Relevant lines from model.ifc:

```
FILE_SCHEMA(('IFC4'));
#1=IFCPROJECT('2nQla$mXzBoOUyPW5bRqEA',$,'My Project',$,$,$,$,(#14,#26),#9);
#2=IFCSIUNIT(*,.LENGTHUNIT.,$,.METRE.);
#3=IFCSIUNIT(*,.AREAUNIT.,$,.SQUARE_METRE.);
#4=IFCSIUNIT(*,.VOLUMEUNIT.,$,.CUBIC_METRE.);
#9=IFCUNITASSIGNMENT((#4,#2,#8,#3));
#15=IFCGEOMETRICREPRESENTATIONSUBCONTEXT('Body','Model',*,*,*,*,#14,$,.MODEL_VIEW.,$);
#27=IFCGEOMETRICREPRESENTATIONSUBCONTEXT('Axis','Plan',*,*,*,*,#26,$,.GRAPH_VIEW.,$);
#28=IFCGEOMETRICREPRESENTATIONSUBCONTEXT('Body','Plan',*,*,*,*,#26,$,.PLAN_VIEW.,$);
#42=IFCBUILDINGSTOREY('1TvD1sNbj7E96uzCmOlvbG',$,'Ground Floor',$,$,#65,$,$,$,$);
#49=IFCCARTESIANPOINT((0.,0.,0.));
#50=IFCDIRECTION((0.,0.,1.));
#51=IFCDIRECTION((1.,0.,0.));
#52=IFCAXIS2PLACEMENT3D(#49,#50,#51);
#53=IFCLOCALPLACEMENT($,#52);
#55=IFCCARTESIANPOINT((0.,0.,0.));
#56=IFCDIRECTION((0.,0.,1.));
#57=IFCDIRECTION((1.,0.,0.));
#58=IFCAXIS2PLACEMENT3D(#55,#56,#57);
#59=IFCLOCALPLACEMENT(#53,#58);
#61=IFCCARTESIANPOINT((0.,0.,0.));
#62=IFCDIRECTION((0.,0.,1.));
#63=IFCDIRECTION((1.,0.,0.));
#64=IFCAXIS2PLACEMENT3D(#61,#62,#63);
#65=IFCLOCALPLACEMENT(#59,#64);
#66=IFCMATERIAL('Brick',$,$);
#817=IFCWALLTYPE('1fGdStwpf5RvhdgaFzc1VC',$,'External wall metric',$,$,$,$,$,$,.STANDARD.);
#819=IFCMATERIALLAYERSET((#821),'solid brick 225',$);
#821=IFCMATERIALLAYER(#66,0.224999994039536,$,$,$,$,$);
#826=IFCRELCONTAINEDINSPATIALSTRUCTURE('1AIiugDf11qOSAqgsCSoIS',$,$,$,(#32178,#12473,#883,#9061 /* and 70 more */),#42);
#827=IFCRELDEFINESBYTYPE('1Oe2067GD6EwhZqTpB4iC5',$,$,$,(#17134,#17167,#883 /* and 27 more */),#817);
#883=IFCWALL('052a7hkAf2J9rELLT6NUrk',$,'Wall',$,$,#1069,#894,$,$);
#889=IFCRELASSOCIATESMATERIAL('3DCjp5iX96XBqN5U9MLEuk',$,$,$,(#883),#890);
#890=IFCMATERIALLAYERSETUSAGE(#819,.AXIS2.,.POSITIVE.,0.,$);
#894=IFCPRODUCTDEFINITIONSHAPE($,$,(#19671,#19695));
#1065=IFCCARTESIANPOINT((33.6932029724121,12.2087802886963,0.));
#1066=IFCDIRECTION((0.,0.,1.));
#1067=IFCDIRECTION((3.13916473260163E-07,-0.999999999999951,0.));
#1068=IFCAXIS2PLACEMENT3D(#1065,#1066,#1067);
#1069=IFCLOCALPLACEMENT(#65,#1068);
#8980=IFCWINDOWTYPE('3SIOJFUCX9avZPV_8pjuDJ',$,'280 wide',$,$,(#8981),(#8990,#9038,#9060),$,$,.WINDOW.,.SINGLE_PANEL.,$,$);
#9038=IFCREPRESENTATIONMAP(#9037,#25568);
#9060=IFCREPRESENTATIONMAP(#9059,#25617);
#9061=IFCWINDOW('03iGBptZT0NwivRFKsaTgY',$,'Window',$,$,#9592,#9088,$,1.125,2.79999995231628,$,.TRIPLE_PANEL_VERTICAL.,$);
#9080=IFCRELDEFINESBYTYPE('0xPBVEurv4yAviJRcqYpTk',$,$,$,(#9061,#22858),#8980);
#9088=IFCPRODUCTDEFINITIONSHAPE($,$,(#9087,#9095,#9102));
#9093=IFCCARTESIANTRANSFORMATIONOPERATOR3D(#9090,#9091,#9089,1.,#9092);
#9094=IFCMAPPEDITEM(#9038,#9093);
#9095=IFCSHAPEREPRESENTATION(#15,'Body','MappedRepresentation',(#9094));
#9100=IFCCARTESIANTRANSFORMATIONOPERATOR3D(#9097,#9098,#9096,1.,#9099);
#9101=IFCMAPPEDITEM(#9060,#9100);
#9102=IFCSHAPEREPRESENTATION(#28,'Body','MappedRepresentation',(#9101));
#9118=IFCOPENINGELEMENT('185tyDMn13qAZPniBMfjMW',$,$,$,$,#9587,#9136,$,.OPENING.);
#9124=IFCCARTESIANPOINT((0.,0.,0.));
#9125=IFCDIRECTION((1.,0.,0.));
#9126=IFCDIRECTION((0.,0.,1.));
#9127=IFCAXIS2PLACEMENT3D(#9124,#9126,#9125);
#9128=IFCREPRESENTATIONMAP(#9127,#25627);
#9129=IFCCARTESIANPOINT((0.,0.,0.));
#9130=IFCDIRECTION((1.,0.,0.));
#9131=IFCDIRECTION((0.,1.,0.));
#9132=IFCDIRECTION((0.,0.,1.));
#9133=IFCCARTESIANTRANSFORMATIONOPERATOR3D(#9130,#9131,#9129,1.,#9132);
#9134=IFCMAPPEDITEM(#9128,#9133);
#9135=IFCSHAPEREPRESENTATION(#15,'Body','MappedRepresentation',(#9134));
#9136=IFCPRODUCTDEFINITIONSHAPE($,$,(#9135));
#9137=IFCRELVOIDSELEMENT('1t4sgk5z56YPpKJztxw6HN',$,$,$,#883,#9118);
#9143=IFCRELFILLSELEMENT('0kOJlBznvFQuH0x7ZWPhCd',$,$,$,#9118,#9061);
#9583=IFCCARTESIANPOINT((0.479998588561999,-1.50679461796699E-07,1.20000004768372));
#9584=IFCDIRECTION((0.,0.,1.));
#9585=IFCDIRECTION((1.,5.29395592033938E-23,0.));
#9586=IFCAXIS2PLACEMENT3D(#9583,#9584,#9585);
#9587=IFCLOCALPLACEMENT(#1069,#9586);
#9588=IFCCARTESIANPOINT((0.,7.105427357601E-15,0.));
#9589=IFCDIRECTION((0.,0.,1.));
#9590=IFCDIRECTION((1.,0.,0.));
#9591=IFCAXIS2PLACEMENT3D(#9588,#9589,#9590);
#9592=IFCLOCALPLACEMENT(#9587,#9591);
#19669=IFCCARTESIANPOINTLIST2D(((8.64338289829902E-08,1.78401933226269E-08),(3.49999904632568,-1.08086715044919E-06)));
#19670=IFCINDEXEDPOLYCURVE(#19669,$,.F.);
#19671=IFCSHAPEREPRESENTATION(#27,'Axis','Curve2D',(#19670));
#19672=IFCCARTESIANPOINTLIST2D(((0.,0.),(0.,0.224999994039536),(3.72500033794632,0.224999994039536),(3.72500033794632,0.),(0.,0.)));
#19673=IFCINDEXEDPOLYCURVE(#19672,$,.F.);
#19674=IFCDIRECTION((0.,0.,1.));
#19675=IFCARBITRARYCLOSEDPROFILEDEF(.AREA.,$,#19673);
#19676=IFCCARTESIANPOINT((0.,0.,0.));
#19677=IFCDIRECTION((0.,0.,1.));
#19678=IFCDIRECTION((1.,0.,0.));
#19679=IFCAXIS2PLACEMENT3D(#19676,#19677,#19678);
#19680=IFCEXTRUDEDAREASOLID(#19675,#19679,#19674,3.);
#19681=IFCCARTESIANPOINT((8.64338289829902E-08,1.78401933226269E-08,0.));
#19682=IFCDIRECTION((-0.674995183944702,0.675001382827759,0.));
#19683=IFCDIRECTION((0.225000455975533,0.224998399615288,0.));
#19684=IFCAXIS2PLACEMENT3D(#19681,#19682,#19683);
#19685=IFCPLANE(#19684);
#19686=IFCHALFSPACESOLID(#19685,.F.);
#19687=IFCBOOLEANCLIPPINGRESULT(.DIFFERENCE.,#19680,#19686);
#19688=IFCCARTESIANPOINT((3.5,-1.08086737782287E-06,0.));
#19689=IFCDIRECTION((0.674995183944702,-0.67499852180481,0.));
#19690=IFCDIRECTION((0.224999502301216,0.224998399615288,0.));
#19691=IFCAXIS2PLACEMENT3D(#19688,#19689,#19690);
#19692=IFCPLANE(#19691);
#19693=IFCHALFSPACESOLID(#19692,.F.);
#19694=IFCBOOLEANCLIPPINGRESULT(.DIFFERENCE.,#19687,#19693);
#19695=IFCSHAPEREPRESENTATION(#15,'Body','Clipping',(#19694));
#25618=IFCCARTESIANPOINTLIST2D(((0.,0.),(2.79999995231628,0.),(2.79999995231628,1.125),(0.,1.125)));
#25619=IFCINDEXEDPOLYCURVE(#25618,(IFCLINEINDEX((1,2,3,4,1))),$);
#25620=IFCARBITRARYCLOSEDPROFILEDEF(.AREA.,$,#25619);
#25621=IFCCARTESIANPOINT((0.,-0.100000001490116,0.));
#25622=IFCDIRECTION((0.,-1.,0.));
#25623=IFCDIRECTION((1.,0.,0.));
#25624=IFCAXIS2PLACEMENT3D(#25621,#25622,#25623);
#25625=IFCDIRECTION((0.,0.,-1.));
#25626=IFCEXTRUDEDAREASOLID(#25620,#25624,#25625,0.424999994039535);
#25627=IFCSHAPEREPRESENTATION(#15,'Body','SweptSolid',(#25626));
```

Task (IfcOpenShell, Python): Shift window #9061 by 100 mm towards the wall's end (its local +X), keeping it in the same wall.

```python
import ifcopenshell
import ifcopenshell.api.geometry
import ifcopenshell.util.placement
import ifcopenshell.util.unit

model = ifcopenshell.open("model.ifc")
unit_scale = ifcopenshell.util.unit.calculate_unit_scale(model)

window = model.by_id(9061)
opening = window.FillsVoids[0].RelatingOpeningElement
wall = opening.VoidsElements[0].RelatingBuildingElement

wall_matrix = ifcopenshell.util.placement.get_local_placement(wall.ObjectPlacement)
shift = wall_matrix[:3, 0] * 0.1 / unit_scale
before = ifcopenshell.util.placement.get_local_placement(window.ObjectPlacement)[:3, 3].copy()

# The window is placed relative to its opening, so it follows when the opening moves.
matrix = ifcopenshell.util.placement.get_local_placement(opening.ObjectPlacement)
matrix[:3, 3] += shift
ifcopenshell.api.geometry.edit_object_placement(
    model, product=opening, matrix=matrix, is_si=False, should_transform_children=True
)

after = ifcopenshell.util.placement.get_local_placement(window.ObjectPlacement)[:3, 3]
print("window moved by", (after - before).round(3) + 0.0)

model.write("model_rev.ifc")
```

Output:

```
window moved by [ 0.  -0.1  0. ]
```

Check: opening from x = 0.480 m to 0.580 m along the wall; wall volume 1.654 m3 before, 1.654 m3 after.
